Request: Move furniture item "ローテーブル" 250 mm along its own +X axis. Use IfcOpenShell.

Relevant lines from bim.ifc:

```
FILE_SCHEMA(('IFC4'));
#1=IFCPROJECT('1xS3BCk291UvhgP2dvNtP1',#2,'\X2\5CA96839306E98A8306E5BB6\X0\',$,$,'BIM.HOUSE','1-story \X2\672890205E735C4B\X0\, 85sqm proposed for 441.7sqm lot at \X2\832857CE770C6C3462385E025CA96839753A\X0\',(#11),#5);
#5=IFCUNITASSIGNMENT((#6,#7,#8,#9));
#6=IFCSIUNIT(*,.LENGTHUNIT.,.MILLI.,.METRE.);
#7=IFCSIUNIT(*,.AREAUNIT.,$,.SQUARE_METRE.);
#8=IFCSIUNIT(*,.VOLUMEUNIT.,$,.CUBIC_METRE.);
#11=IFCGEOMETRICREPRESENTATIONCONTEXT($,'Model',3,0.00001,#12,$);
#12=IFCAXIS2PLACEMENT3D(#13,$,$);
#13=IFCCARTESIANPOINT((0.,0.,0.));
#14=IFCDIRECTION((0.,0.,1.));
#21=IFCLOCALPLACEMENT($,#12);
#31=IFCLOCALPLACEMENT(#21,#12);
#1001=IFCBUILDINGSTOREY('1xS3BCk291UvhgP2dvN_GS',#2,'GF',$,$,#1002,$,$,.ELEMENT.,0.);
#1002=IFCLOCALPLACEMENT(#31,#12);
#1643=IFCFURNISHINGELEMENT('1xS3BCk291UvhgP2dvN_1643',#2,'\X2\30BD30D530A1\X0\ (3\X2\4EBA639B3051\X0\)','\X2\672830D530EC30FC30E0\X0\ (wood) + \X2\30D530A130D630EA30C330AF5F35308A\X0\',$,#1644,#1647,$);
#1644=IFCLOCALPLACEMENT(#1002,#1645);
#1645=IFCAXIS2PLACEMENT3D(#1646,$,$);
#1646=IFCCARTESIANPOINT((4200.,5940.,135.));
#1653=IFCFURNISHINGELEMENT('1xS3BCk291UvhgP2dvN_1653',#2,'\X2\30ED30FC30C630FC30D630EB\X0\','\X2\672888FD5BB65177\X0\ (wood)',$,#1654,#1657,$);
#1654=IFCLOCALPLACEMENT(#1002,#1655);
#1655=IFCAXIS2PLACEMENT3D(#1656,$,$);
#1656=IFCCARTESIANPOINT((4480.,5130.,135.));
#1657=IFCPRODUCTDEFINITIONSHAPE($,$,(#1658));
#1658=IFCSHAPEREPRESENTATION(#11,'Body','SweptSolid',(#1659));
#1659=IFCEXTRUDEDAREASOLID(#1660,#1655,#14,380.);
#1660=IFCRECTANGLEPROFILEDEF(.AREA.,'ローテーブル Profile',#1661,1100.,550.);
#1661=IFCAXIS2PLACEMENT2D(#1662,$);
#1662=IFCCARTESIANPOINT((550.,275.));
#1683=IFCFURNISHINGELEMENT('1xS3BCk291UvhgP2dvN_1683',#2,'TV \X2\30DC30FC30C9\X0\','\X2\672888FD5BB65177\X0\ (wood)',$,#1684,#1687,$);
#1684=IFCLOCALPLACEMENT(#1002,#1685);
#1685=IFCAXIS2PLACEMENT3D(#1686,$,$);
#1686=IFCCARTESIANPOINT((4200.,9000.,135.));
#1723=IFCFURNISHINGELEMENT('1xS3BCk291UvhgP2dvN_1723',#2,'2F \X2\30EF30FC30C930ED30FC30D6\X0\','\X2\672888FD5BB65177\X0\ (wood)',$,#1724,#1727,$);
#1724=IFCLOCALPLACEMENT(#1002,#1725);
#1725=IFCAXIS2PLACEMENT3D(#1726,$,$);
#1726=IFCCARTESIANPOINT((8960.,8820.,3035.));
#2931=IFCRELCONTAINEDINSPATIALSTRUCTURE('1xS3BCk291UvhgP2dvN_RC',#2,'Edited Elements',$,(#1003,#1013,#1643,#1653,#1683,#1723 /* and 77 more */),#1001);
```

```python
import ifcopenshell
import ifcopenshell.api.geometry
import ifcopenshell.util.placement

model = ifcopenshell.open("bim.ifc")

item = model.by_guid("1xS3BCk291UvhgP2dvN_1653")
matrix = ifcopenshell.util.placement.get_local_placement(item.ObjectPlacement)
matrix[:3, 3] += matrix[:3, 0] * 250.0
ifcopenshell.api.geometry.edit_object_placement(model, product=item, matrix=matrix, is_si=False)

print(ifcopenshell.util.placement.get_local_placement(item.ObjectPlacement).round(3) + 0.0)

model.write("bim_rev.ifc")
```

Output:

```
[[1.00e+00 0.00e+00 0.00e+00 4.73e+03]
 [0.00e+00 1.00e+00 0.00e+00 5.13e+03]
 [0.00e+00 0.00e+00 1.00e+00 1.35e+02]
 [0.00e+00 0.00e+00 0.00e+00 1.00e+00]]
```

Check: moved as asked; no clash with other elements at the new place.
